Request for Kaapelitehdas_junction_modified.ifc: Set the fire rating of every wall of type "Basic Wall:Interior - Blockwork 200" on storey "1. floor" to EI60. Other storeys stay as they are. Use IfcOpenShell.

First a look at what the model holds.

```python
import ifcopenshell
import ifcopenshell.util.element

model = ifcopenshell.open("Kaapelitehdas_junction_modified.ifc")
print(model.schema)
storey = next(s for s in model.by_type("IfcBuildingStorey") if s.Name == "1. floor")
walls = [e for e in ifcopenshell.util.element.get_decomposition(storey) if e.is_a("IfcWall")]
seen = {}
for e in walls:
    element_type = ifcopenshell.util.element.get_type(e)
    key = (element_type.Name if element_type != e and element_type else None, ifcopenshell.util.element.get_pset(e, "Pset_WallCommon", "FireRating"))
    seen[key] = seen.get(key, 0) + 1
for (name, value), count in sorted(seen.items(), key=str):
    print(count, "x", name, "|", value)
```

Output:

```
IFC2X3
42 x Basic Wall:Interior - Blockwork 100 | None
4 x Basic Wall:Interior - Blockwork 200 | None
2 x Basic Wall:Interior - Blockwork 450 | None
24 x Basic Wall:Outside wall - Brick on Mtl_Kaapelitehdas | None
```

```python
import ifcopenshell
import ifcopenshell.api.pset
import ifcopenshell.util.element

model = ifcopenshell.open("Kaapelitehdas_junction_modified.ifc")

storey = next(s for s in model.by_type("IfcBuildingStorey") if s.Name == "1. floor")
walls = [e for e in ifcopenshell.util.element.get_decomposition(storey) if e.is_a("IfcWall")]

count = 0
for e in walls:
    element_type = ifcopenshell.util.element.get_type(e)
    if element_type in (None, e) or element_type.Name != "Basic Wall:Interior - Blockwork 200":
        continue
    # add_pset returns the element's existing set when there is one.
    pset = ifcopenshell.api.pset.add_pset(model, product=e, name="Pset_WallCommon")
    ifcopenshell.api.pset.edit_pset(model, pset=pset, properties={"FireRating": "EI60"})
    count += 1

print(count, "walls updated")

model.write("Kaapelitehdas_junction_modified_rev.ifc")
```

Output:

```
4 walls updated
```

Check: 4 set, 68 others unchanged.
